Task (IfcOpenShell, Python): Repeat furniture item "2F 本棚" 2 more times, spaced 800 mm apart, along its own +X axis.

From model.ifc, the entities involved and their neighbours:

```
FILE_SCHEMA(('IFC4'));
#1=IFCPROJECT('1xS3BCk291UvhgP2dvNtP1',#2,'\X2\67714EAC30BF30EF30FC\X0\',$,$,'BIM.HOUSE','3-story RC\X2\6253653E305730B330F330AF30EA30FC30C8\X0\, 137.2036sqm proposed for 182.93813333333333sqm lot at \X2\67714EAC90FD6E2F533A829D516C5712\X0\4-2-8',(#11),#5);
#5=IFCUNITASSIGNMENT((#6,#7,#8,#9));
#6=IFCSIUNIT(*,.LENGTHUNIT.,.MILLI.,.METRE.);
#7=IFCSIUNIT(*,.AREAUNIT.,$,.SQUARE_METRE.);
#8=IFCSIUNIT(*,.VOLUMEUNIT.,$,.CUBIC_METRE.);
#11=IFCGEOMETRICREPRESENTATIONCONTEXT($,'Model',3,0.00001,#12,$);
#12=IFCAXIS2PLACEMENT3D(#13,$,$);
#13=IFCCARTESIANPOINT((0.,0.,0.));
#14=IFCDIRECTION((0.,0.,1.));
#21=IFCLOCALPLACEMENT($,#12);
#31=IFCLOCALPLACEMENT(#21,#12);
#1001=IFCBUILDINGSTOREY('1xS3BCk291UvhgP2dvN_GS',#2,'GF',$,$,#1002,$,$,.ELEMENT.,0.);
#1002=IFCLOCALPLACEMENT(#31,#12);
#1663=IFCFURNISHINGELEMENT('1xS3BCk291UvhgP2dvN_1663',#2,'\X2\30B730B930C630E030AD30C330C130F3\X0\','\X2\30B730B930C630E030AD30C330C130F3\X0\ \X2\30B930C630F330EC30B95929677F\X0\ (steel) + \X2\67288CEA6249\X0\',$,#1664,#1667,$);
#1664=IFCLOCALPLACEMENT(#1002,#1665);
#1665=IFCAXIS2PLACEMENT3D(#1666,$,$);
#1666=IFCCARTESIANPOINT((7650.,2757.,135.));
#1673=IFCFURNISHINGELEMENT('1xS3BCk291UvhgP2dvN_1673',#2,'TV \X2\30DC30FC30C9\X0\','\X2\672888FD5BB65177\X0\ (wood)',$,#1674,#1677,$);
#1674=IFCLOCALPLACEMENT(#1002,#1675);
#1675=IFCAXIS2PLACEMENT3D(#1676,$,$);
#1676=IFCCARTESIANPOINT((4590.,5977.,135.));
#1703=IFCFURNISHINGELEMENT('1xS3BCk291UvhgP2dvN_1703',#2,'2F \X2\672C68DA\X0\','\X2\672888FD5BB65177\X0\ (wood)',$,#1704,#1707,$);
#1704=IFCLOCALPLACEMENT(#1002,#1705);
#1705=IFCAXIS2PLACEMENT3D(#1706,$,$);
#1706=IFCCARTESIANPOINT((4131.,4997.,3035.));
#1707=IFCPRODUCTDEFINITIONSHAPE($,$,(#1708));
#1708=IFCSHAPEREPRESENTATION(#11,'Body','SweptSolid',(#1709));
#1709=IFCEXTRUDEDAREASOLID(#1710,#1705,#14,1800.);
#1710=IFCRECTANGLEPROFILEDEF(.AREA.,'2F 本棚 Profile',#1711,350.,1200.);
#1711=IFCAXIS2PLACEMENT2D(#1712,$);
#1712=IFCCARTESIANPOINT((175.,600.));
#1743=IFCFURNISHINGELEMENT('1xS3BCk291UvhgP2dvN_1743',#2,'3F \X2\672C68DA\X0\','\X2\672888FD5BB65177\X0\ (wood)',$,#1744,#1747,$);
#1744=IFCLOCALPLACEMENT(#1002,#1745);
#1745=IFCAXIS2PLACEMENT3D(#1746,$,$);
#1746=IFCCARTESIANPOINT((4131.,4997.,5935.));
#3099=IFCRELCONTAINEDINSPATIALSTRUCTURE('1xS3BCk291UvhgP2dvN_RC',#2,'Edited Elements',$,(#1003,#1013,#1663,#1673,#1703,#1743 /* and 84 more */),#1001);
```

```python
import ifcopenshell
import ifcopenshell.api.geometry
import ifcopenshell.api.root
import ifcopenshell.util.element
import ifcopenshell.util.placement
import ifcopenshell.util.unit

model = ifcopenshell.open("model.ifc")
unit_scale = ifcopenshell.util.unit.calculate_unit_scale(model)


def reuse_history(source, copy):
    """copy_class also copies each property set's owner history, people and application; keep the originals."""
    for rel in copy.IsDefinedBy:
        if rel.is_a("IfcRelDefinesByProperties") and (history := rel.RelatingPropertyDefinition.OwnerHistory):
            rel.RelatingPropertyDefinition.OwnerHistory = source.OwnerHistory
            ifcopenshell.util.element.remove_deep2(model, history)


source = model.by_id(1703)
base = ifcopenshell.util.placement.get_local_placement(source.ObjectPlacement)
step = base[:3, 0] * 0.8 / unit_scale

for i in range(1, 3):
    copy = ifcopenshell.api.root.copy_class(model, product=source)
    copy.Representation = ifcopenshell.util.element.copy_deep(
        model, source.Representation, exclude=["IfcGeometricRepresentationContext", "IfcRepresentationMap"]
    )
    reuse_history(source, copy)
    matrix = base.copy()
    matrix[:3, 3] += i * step
    print("added at", matrix[:3, 3].round(3) + 0.0)
    ifcopenshell.api.geometry.edit_object_placement(model, product=copy, matrix=matrix, is_si=False)

model.write("model_edited.ifc")
```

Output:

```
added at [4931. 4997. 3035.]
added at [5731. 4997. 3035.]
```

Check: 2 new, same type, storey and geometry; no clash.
